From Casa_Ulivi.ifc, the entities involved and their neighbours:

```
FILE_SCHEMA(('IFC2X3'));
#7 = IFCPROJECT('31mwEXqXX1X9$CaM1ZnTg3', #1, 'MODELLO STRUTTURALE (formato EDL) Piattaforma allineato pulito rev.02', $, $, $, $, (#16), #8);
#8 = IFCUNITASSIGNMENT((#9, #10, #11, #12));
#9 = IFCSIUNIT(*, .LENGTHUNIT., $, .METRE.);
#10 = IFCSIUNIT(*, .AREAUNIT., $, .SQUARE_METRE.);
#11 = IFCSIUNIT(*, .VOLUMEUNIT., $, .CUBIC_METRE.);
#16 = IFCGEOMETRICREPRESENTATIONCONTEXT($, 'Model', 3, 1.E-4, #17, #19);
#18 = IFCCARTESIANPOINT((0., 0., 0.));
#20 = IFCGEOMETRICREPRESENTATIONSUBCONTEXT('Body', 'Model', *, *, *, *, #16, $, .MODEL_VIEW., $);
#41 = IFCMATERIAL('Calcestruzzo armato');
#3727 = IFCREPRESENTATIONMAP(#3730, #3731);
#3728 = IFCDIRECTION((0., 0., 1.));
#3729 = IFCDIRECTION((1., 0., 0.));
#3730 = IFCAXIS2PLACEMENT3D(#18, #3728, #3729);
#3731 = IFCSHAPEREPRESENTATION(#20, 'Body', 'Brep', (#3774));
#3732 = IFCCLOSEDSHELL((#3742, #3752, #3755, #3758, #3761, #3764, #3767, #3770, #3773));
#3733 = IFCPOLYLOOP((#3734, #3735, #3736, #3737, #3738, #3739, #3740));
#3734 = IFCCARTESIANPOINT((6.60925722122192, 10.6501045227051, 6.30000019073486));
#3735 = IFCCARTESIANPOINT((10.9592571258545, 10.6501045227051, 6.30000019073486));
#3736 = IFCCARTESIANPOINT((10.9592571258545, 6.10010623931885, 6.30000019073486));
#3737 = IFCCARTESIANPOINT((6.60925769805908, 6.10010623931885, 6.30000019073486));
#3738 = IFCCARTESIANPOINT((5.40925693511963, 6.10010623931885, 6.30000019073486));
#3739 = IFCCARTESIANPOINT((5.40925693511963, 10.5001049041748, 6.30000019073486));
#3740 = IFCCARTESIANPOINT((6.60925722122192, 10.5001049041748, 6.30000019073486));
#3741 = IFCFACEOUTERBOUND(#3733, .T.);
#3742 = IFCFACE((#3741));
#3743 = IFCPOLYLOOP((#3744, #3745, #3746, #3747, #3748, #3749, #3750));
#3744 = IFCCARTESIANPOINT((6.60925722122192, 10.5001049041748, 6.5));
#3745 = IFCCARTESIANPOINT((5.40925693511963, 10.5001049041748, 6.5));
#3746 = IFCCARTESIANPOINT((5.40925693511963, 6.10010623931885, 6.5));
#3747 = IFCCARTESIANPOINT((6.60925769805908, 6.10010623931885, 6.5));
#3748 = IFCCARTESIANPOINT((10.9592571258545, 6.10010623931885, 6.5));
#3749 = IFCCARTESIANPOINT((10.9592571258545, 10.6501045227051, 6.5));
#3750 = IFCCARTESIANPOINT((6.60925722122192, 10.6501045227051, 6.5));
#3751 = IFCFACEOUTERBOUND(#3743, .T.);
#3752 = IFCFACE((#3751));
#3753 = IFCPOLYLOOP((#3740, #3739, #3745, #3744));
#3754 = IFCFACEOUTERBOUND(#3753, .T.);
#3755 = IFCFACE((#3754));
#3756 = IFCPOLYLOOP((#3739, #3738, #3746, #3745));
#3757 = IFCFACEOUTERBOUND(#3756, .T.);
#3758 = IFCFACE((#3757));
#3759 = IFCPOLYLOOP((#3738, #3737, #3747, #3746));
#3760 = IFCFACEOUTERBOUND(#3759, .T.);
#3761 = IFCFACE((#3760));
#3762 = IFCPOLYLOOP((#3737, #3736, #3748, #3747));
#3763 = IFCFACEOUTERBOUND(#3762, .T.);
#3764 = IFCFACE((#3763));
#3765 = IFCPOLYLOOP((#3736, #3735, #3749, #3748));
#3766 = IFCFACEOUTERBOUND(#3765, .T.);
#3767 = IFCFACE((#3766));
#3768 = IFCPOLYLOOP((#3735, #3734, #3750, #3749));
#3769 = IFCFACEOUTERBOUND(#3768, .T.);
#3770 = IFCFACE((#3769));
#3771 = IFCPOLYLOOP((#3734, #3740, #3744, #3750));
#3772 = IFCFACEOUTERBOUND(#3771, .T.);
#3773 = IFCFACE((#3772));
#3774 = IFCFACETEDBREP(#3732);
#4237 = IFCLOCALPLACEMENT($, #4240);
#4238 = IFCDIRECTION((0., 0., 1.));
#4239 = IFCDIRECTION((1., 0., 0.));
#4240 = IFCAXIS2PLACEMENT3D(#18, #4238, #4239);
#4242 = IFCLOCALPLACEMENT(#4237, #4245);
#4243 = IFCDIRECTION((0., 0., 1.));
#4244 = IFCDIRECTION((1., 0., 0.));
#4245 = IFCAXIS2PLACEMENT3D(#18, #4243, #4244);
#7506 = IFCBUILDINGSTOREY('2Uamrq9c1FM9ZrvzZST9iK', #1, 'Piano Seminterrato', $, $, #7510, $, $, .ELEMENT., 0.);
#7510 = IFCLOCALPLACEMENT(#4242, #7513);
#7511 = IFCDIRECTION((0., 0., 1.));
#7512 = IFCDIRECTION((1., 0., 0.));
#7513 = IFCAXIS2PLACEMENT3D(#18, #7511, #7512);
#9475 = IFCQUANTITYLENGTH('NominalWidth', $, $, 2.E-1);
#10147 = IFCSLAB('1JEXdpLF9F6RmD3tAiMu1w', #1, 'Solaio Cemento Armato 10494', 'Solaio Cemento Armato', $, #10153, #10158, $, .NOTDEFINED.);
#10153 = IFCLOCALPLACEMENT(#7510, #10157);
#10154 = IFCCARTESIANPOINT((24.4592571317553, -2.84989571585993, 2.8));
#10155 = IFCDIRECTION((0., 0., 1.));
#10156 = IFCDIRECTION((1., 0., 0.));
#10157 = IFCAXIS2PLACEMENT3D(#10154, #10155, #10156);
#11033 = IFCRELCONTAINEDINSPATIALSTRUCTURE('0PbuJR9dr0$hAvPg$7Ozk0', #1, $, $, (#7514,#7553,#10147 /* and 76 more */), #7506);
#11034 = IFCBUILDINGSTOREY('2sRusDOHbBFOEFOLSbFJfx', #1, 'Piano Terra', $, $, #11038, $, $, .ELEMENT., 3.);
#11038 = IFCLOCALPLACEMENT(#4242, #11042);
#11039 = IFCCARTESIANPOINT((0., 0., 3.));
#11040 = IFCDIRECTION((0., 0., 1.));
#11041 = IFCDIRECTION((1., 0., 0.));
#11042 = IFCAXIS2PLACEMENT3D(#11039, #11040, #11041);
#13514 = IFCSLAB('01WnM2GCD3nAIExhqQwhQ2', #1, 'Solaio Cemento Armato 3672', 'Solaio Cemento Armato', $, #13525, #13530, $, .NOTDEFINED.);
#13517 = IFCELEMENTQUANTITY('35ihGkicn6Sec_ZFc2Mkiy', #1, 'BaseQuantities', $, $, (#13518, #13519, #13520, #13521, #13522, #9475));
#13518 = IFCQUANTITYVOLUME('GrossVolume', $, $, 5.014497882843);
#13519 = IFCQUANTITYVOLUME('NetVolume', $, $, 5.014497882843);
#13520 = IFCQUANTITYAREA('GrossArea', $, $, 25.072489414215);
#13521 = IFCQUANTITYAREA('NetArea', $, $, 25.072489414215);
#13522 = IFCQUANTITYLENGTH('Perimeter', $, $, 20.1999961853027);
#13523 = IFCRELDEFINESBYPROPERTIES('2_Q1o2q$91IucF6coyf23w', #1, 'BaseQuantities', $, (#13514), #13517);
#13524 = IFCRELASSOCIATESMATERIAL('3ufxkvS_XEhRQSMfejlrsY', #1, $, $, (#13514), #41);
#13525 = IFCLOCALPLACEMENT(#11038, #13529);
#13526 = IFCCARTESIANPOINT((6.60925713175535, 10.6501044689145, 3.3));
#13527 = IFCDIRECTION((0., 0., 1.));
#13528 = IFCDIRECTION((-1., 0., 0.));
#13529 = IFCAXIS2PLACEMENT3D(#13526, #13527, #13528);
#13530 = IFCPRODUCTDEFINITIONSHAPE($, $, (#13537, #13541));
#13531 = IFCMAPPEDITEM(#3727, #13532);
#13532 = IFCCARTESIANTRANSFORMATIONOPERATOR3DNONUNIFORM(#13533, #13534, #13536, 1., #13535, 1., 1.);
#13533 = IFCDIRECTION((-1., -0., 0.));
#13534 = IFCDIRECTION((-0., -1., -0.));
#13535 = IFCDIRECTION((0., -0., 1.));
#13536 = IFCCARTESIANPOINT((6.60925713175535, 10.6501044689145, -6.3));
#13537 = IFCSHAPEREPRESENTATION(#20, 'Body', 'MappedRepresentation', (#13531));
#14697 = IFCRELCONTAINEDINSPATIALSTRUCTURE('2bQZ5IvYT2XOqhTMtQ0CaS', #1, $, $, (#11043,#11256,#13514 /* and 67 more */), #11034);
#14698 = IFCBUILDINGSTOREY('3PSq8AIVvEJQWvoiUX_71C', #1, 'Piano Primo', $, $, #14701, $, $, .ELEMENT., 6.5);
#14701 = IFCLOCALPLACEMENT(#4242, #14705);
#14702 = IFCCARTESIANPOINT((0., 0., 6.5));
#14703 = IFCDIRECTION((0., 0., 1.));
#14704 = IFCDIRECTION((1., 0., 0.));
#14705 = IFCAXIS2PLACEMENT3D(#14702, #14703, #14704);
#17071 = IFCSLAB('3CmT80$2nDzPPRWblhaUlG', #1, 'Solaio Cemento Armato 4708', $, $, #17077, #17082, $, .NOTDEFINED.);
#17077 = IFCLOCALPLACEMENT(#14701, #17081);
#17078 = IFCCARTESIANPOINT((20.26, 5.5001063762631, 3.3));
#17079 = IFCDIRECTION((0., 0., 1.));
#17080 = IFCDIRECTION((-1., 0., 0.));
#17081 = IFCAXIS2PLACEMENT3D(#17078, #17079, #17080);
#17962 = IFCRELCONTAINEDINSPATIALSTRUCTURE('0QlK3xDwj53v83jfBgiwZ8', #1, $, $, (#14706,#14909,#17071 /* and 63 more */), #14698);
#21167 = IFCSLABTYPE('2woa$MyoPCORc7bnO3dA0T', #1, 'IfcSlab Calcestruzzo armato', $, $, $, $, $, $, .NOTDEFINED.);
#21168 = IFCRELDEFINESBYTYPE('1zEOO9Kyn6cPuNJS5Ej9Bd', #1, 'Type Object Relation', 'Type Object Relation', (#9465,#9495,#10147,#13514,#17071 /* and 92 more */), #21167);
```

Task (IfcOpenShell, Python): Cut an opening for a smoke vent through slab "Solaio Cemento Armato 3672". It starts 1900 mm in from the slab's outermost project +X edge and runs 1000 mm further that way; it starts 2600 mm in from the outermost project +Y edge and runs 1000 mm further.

```python
import numpy as np
import ifcopenshell
import ifcopenshell.api.feature
import ifcopenshell.api.geometry
import ifcopenshell.api.pset
import ifcopenshell.api.root
import ifcopenshell.geom
import ifcopenshell.util.element
import ifcopenshell.util.placement
import ifcopenshell.util.representation
import ifcopenshell.util.shape
import ifcopenshell.util.unit

model = ifcopenshell.open("Casa_Ulivi.ifc")
unit_scale = ifcopenshell.util.unit.calculate_unit_scale(model)
area_scale = ifcopenshell.util.unit.calculate_unit_scale(model, "AREAUNIT")
volume_scale = ifcopenshell.util.unit.calculate_unit_scale(model, "VOLUMEUNIT")
settings = ifcopenshell.geom.settings()


def volume(element):
    """Net volume in cubic metres, openings subtracted."""
    shape = ifcopenshell.geom.create_shape(settings, element)
    return ifcopenshell.util.shape.get_volume(shape.geometry)


slab = model.by_guid("01WnM2GCD3nAIExhqQwhQ2")
before = volume(slab)

# Extent in the slab's own axes, in metres. The edges named are its -X and -Y sides.
slab_shape = ifcopenshell.geom.create_shape(settings, slab)
vertices = ifcopenshell.util.shape.get_vertices(slab_shape.geometry)
x_min, y_min, bottom = vertices.min(axis=0)
top = vertices[:, 2].max()

opening = ifcopenshell.api.root.create_entity(model, ifc_class="IfcOpeningElement", name="Smoke vent opening")
context = ifcopenshell.util.representation.get_context(model, "Model", "Body", "MODEL_VIEW")
width, depth = 1, 1
outline = [(0.0, 0.0), (width, 0.0), (width, depth), (0.0, depth), (0.0, 0.0)]
# Overshoot both faces by 50 mm so the cut is clean.
shape = ifcopenshell.api.geometry.add_slab_representation(
    model, context=context, depth=top - bottom + 0.1, polyline=outline
)
ifcopenshell.api.geometry.assign_representation(model, product=opening, representation=shape)

matrix = ifcopenshell.util.placement.get_local_placement(slab.ObjectPlacement)
matrix[:, 3] = matrix @ np.append(np.array([x_min + 1.9, y_min + 2.6, bottom - 0.05]) / unit_scale, 1.0)
ifcopenshell.api.geometry.edit_object_placement(model, product=opening, matrix=matrix, is_si=False)
ifcopenshell.api.feature.add_feature(model, feature=opening, element=slab)

after = volume(slab)

# Update the slab's stored quantities.
qto = model.by_id(ifcopenshell.util.element.get_pset(slab, "BaseQuantities", should_inherit=False)["id"])
ifcopenshell.api.pset.edit_qto(model, qto=qto, properties={
    "NetVolume": after / volume_scale,
    "NetArea": after / (top - bottom) / area_scale,
})

print(f"slab volume {before:.3f} -> {after:.3f} m3")

model.write("Casa_Ulivi_updated.ifc")
```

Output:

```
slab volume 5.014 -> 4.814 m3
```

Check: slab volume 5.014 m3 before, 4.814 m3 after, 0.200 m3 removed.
